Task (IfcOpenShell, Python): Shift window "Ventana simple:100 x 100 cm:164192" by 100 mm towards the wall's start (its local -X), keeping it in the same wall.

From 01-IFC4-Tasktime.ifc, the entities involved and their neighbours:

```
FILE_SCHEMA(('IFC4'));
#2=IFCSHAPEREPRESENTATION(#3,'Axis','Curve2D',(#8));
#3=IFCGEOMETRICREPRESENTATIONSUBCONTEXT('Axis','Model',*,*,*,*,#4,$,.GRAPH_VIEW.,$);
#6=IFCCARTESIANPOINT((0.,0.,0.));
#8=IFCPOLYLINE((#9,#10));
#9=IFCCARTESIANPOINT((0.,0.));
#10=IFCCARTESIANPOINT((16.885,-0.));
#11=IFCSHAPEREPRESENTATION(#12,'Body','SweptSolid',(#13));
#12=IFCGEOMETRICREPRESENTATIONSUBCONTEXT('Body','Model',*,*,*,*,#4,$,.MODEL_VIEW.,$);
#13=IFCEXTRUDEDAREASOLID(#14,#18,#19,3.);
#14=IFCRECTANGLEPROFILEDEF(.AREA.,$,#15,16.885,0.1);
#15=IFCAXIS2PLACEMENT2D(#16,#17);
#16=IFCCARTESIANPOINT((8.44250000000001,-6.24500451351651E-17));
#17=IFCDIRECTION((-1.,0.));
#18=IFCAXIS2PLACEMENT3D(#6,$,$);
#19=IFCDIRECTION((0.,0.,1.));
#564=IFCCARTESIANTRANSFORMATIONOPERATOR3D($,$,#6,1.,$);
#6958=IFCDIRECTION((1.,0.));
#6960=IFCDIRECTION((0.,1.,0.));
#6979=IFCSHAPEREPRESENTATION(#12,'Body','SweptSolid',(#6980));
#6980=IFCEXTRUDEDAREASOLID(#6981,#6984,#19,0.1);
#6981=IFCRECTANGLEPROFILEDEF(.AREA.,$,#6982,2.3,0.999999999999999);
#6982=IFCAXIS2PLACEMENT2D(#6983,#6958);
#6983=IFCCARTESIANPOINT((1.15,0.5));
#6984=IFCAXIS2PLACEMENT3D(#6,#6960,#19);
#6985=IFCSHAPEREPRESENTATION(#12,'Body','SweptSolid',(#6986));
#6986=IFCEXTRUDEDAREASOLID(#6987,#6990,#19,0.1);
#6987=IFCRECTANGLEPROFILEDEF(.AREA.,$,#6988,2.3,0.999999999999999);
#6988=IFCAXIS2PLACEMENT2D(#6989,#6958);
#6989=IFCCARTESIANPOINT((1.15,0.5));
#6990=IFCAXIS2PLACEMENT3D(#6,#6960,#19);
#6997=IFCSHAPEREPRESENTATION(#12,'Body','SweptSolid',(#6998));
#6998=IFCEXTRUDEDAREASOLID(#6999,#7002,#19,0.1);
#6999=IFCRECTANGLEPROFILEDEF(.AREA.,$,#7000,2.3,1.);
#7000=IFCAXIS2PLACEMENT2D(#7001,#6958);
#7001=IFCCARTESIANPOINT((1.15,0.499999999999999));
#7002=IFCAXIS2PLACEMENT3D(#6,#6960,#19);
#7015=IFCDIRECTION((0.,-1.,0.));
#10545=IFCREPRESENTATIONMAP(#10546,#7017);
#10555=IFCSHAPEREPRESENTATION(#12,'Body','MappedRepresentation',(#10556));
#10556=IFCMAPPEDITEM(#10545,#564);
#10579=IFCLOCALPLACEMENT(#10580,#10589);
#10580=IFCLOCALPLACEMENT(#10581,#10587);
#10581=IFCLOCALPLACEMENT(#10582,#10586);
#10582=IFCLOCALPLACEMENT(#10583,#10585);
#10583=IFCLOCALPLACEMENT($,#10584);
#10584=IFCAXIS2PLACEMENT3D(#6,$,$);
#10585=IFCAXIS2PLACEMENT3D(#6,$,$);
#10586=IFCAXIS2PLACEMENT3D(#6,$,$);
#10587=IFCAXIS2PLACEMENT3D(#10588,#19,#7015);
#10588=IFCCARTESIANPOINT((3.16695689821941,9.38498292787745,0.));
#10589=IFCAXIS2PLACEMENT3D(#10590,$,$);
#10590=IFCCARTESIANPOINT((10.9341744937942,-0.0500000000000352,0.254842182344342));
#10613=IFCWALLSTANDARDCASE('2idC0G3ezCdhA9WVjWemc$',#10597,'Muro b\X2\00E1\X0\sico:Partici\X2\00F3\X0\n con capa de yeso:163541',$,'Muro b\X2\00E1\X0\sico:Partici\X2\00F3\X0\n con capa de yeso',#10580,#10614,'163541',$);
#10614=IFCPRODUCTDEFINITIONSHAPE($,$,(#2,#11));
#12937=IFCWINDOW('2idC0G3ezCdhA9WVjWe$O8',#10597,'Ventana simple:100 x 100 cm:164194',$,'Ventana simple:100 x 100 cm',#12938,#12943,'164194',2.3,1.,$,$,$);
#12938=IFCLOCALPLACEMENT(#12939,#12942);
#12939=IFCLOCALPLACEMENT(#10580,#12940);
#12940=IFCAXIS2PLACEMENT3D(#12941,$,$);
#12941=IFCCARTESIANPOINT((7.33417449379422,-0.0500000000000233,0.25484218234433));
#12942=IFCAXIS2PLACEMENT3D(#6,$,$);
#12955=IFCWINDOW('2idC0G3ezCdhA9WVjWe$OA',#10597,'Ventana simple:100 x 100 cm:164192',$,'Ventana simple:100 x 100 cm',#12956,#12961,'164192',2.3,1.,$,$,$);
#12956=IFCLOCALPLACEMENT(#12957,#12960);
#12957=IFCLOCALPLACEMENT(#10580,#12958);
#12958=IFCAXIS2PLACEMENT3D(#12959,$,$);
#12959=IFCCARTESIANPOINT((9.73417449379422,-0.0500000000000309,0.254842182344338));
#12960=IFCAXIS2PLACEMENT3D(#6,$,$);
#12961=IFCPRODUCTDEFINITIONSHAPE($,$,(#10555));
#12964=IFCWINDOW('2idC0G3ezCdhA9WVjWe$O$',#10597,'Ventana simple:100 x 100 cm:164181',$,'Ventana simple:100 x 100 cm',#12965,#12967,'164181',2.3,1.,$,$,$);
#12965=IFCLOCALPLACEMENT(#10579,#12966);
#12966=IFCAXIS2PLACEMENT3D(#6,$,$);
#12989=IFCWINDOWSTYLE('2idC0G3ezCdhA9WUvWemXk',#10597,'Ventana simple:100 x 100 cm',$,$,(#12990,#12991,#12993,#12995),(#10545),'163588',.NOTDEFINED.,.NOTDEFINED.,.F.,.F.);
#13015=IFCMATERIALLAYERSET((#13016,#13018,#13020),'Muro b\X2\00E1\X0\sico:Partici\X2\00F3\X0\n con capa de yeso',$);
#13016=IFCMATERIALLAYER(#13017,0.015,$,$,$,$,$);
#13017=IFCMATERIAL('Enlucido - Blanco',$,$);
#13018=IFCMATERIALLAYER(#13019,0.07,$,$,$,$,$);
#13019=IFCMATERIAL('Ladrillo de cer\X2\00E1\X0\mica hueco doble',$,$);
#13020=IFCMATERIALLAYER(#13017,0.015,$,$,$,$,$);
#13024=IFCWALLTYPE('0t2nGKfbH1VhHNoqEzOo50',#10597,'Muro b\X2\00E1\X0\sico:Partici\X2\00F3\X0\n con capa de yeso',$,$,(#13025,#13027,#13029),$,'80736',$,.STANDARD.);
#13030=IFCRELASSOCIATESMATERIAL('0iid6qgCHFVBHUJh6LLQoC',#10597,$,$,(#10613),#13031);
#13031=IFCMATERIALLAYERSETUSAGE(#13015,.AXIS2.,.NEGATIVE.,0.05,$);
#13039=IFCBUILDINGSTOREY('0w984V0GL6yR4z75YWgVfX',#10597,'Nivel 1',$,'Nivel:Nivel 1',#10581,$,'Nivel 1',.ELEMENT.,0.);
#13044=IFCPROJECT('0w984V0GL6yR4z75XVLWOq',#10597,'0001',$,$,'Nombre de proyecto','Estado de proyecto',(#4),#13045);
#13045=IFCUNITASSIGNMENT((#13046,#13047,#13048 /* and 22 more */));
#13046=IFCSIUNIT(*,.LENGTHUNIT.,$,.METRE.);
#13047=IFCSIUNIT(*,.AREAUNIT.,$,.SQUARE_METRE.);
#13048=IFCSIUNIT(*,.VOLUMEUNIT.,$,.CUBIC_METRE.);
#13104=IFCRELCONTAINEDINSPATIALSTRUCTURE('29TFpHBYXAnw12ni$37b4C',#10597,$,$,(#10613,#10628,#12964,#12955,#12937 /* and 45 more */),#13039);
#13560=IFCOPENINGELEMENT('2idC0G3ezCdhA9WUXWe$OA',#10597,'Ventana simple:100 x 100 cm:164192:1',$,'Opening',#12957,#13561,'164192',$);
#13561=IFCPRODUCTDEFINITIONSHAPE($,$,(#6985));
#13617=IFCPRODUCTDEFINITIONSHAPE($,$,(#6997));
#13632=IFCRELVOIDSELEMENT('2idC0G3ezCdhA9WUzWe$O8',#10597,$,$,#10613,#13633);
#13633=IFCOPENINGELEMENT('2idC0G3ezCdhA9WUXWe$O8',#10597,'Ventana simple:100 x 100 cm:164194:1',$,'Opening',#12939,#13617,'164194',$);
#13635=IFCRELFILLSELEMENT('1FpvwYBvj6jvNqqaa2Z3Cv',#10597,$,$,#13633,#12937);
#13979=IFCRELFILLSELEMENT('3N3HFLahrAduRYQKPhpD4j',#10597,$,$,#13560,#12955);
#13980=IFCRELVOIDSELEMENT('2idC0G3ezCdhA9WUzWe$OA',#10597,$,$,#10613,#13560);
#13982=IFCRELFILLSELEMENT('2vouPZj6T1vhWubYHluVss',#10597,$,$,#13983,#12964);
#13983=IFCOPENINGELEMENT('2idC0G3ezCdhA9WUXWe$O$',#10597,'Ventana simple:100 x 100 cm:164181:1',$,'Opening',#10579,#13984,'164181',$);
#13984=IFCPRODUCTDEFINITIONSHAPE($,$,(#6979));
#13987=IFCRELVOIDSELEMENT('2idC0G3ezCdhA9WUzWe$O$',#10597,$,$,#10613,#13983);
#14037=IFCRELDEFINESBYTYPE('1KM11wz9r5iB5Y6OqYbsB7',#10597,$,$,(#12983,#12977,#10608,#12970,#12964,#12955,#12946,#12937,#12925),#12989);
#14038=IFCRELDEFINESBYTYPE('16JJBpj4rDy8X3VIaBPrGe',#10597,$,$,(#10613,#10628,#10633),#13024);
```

```python
import ifcopenshell
import ifcopenshell.api.geometry
import ifcopenshell.util.placement
import ifcopenshell.util.unit

model = ifcopenshell.open("01-IFC4-Tasktime.ifc")
unit_scale = ifcopenshell.util.unit.calculate_unit_scale(model)

window = model.by_guid("2idC0G3ezCdhA9WVjWe$OA")
opening = window.FillsVoids[0].RelatingOpeningElement
wall = opening.VoidsElements[0].RelatingBuildingElement

wall_matrix = ifcopenshell.util.placement.get_local_placement(wall.ObjectPlacement)
shift = wall_matrix[:3, 0] * -0.1 / unit_scale
before = ifcopenshell.util.placement.get_local_placement(window.ObjectPlacement)[:3, 3].copy()

# The window is placed relative to its opening, so it follows when the opening moves.
matrix = ifcopenshell.util.placement.get_local_placement(opening.ObjectPlacement)
matrix[:3, 3] += shift
ifcopenshell.api.geometry.edit_object_placement(
    model, product=opening, matrix=matrix, is_si=False, should_transform_children=True
)

after = ifcopenshell.util.placement.get_local_placement(window.ObjectPlacement)[:3, 3]
print("window moved by", (after - before).round(3) + 0.0)

model.write("01-IFC4-Tasktime-out.ifc")
```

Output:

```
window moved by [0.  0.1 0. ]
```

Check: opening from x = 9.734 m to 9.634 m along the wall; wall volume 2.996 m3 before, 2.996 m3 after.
